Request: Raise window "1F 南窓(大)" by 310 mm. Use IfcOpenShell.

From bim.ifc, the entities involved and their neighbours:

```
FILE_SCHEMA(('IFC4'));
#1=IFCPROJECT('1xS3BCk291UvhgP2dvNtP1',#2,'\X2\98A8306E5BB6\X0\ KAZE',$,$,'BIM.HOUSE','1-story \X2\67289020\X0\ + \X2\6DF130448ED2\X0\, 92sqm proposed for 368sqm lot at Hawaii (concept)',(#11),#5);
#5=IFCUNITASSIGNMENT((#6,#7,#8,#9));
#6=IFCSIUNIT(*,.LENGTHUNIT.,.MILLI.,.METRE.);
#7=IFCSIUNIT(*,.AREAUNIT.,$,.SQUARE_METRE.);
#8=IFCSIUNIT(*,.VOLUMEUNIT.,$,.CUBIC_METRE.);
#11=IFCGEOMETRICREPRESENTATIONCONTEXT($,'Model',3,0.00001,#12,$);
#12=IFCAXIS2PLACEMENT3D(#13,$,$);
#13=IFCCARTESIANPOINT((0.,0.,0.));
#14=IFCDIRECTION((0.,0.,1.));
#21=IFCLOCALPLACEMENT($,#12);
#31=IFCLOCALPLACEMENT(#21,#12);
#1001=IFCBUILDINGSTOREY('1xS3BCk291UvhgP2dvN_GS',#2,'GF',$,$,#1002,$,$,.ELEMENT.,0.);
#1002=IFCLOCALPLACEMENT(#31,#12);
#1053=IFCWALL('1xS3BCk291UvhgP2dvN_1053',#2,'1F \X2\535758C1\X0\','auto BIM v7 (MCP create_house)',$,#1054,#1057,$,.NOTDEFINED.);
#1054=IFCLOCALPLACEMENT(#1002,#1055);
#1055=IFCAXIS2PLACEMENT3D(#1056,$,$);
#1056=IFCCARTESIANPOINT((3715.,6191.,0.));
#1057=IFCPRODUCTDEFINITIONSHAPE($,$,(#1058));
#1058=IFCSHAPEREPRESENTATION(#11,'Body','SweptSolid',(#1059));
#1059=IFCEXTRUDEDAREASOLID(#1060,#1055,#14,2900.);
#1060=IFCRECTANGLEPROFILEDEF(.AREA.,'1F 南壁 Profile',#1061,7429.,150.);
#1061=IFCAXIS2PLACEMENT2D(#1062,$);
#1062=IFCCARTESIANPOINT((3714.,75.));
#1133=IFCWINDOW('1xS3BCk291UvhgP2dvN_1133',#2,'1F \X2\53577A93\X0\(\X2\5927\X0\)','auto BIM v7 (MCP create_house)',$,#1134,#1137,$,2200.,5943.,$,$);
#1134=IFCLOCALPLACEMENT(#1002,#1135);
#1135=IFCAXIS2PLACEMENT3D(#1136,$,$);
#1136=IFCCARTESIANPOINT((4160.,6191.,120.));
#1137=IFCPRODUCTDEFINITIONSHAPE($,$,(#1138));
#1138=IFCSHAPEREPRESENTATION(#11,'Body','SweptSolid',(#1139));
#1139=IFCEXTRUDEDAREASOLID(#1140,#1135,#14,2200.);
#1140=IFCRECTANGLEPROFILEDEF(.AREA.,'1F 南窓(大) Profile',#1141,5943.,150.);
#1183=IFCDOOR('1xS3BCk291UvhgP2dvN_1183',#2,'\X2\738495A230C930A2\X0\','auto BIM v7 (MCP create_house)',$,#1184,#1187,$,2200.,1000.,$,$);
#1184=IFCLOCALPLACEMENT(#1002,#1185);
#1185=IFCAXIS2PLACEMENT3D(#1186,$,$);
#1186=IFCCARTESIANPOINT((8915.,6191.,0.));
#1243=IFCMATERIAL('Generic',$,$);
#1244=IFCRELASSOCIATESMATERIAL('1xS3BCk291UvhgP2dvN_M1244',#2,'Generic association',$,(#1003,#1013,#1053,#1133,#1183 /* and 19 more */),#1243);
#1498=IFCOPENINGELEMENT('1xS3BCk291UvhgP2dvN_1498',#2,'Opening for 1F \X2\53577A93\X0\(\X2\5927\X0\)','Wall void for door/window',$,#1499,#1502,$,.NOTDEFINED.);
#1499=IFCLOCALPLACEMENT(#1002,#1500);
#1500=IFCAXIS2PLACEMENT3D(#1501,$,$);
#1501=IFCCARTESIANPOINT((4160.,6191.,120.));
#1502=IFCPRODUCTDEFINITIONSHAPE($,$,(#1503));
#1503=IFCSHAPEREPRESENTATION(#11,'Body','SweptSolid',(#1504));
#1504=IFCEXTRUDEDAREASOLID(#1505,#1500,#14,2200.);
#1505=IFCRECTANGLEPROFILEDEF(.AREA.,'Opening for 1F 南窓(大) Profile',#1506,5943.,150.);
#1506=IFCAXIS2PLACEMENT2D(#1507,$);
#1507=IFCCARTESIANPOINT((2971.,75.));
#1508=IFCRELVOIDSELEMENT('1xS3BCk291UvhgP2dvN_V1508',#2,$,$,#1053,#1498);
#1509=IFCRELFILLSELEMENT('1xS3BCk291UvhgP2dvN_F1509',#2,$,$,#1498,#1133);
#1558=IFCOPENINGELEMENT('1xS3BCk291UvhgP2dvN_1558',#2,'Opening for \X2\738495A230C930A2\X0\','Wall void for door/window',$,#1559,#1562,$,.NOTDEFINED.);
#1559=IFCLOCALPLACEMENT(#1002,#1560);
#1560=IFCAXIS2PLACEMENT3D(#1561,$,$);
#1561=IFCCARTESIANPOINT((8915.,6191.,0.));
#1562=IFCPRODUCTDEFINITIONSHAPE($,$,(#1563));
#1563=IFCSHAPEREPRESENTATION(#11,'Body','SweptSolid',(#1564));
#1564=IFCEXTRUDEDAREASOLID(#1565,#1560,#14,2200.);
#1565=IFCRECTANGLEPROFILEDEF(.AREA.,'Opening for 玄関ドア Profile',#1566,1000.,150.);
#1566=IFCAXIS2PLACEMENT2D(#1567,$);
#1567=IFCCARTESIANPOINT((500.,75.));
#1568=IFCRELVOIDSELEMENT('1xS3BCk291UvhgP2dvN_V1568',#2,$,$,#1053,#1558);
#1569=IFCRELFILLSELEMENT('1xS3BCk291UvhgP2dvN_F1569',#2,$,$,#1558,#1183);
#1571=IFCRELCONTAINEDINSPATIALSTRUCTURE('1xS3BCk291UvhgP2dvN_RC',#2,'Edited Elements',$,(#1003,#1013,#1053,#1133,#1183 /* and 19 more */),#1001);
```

```python
import numpy as np
import ifcopenshell
import ifcopenshell.api.geometry
import ifcopenshell.util.placement
import ifcopenshell.util.unit

model = ifcopenshell.open("bim.ifc")
unit_scale = ifcopenshell.util.unit.calculate_unit_scale(model)

window = model.by_guid("1xS3BCk291UvhgP2dvN_1133")
opening = window.FillsVoids[0].RelatingOpeningElement
dz = 0.31 / unit_scale

shift = np.array([0.0, 0.0, dz])
# The window is not placed relative to its opening, so move both.
for product in (opening, window):
    matrix = ifcopenshell.util.placement.get_local_placement(product.ObjectPlacement)
    matrix[:3, 3] += shift
    ifcopenshell.api.geometry.edit_object_placement(model, product=product, matrix=matrix, is_si=False)

print(f"moved by {dz * unit_scale:+.3f} m")

model.write("bim_rev.ifc")
```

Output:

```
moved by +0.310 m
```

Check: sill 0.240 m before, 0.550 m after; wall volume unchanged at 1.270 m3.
